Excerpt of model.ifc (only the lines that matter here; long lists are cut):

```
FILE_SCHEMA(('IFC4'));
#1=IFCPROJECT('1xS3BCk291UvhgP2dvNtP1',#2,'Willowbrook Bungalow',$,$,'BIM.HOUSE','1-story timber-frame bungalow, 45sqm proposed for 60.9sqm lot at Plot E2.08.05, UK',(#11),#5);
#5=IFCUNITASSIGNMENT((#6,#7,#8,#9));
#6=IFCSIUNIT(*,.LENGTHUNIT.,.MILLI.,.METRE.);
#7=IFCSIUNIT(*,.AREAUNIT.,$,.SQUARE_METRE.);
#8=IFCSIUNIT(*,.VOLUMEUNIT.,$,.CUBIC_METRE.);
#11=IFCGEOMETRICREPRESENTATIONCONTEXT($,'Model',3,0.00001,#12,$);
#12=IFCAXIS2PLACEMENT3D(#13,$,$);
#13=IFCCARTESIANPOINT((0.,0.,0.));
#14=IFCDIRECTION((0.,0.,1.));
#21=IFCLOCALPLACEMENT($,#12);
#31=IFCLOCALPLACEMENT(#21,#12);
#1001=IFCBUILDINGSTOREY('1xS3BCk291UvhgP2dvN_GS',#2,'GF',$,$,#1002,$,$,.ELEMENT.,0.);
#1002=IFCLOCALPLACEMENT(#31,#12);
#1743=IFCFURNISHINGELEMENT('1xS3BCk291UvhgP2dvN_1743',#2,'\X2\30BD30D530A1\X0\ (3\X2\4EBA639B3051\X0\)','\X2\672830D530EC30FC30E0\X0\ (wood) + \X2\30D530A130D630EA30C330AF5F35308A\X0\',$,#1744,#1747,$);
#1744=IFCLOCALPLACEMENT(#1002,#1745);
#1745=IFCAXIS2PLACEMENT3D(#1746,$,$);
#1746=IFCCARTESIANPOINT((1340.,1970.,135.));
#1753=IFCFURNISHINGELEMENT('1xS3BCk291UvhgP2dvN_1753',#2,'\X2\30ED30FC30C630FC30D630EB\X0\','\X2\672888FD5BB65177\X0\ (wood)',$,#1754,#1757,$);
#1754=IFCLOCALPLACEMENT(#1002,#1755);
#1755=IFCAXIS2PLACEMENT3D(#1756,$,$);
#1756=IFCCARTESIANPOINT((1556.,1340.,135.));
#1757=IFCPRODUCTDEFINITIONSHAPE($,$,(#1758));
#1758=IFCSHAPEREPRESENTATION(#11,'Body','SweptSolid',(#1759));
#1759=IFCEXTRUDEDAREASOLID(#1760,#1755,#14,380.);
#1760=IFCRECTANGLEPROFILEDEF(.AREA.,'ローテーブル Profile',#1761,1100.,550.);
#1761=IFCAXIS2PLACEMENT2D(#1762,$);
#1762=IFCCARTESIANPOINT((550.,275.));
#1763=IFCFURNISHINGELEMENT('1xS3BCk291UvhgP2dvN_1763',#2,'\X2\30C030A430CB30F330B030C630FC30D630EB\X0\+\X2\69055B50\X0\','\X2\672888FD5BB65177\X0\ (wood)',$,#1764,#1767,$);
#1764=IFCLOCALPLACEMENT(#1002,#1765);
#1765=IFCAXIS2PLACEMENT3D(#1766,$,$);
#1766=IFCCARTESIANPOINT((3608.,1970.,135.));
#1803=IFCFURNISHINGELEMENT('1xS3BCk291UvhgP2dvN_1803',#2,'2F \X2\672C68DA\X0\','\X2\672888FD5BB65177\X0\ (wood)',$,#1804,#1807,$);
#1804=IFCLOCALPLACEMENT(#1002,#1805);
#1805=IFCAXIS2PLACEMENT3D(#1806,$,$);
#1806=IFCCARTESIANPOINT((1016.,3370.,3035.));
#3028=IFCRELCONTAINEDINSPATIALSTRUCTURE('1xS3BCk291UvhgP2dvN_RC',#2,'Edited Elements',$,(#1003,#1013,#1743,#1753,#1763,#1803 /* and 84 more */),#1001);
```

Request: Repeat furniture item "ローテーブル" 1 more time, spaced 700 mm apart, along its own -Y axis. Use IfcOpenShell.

```python
import ifcopenshell
import ifcopenshell.api.geometry
import ifcopenshell.api.root
import ifcopenshell.util.element
import ifcopenshell.util.placement

model = ifcopenshell.open("model.ifc")


def reuse_history(source, copy):
    """copy_class also copies each property set's owner history, people and application; keep the originals."""
    for rel in copy.IsDefinedBy:
        if rel.is_a("IfcRelDefinesByProperties") and (history := rel.RelatingPropertyDefinition.OwnerHistory):
            rel.RelatingPropertyDefinition.OwnerHistory = source.OwnerHistory
            ifcopenshell.util.element.remove_deep2(model, history)


source = model.by_guid("1xS3BCk291UvhgP2dvN_1753")
base = ifcopenshell.util.placement.get_local_placement(source.ObjectPlacement)
step = -base[:3, 1] * 700.0

for i in range(1, 2):
    copy = ifcopenshell.api.root.copy_class(model, product=source)
    copy.Representation = ifcopenshell.util.element.copy_deep(
        model, source.Representation, exclude=["IfcGeometricRepresentationContext", "IfcRepresentationMap"]
    )
    reuse_history(source, copy)
    matrix = base.copy()
    matrix[:3, 3] += i * step
    print("added at", matrix[:3, 3].round(3) + 0.0)
    ifcopenshell.api.geometry.edit_object_placement(model, product=copy, matrix=matrix, is_si=False)

model.write("model_updated.ifc")
```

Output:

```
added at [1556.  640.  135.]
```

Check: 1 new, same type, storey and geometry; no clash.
